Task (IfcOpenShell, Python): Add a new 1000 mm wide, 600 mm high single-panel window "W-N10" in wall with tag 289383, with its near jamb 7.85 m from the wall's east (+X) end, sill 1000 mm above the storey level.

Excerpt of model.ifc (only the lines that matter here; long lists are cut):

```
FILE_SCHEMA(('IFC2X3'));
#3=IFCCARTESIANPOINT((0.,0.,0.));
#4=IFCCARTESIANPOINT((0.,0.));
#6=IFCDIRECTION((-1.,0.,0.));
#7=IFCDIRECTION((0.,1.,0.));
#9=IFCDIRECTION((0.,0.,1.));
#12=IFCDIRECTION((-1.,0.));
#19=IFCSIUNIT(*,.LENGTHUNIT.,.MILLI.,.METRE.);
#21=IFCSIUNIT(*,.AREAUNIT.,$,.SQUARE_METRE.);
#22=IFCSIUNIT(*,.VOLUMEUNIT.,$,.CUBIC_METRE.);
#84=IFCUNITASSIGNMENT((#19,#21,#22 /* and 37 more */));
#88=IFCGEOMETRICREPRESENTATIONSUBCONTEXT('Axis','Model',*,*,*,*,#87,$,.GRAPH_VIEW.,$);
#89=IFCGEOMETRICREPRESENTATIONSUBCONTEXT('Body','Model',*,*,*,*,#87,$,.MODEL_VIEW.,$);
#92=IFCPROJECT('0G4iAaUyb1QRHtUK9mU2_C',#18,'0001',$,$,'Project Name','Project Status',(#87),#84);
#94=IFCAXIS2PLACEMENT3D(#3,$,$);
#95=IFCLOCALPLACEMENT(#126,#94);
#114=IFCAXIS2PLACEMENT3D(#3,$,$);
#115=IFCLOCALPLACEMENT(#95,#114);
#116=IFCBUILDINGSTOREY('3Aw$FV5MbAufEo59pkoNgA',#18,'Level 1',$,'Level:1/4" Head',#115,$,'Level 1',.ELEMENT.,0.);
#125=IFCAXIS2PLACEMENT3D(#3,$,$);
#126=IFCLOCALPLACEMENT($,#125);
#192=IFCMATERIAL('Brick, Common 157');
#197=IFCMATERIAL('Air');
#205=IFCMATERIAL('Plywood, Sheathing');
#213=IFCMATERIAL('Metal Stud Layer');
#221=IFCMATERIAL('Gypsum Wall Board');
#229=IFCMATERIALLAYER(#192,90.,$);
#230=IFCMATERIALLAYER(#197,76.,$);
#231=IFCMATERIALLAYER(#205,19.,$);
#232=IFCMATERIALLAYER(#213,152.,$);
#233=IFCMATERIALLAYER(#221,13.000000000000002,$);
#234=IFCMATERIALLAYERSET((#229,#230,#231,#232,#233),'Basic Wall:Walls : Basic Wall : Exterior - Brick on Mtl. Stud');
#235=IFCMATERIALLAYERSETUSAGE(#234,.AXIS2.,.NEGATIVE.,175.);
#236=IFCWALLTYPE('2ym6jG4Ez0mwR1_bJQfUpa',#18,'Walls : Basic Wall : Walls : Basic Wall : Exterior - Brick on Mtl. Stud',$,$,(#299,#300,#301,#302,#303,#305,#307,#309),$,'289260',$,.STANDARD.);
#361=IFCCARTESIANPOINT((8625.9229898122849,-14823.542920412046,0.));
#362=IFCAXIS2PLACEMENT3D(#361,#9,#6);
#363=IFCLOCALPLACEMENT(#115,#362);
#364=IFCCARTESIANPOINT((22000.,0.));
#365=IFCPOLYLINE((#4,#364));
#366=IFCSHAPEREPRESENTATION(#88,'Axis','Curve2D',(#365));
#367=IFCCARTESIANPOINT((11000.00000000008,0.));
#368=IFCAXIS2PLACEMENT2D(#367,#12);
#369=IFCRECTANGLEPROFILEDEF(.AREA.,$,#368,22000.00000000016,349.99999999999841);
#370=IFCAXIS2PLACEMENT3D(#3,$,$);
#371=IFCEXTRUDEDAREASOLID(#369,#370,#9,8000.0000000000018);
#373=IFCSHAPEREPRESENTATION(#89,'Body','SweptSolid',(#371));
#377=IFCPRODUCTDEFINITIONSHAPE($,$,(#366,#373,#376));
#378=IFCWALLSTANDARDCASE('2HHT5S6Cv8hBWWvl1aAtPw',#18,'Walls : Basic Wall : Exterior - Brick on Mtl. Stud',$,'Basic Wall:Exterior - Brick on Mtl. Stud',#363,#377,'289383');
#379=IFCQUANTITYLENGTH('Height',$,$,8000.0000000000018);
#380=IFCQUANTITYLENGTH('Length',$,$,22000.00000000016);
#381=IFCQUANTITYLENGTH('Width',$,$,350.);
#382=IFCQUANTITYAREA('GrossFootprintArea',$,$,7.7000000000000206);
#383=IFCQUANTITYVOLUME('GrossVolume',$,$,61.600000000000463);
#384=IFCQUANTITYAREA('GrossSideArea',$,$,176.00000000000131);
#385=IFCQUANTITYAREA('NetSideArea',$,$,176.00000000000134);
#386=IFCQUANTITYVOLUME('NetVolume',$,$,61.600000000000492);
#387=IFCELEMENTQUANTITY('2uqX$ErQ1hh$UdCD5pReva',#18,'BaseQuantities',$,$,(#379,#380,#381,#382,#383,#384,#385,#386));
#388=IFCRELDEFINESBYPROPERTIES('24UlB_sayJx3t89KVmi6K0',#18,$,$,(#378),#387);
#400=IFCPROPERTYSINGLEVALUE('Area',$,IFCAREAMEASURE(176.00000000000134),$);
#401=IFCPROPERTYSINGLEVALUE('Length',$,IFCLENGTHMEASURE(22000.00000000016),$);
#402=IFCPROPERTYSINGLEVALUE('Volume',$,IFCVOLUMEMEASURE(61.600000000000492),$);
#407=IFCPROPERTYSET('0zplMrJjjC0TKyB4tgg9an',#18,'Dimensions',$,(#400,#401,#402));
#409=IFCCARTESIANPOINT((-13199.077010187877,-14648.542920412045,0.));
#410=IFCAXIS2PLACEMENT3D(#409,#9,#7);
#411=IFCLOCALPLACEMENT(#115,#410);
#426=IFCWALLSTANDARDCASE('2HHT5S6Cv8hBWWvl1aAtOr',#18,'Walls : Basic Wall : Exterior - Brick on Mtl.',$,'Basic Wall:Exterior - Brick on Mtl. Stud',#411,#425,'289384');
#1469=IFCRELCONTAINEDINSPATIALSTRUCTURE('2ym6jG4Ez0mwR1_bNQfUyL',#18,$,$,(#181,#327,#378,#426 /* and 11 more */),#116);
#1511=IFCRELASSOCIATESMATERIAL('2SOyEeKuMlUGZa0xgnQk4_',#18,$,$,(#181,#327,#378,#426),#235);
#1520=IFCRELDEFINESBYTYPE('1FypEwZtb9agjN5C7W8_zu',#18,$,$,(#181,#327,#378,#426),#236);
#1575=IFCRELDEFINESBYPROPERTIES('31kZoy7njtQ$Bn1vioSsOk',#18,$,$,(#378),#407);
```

```python
import numpy as np
import ifcopenshell
import ifcopenshell.api.feature
import ifcopenshell.api.geometry
import ifcopenshell.api.pset
import ifcopenshell.api.root
import ifcopenshell.api.spatial
import ifcopenshell.api.type
import ifcopenshell.geom
import ifcopenshell.util.element
import ifcopenshell.util.placement
import ifcopenshell.util.representation
import ifcopenshell.util.shape
import ifcopenshell.util.unit

model = ifcopenshell.open("model.ifc")
unit_scale = ifcopenshell.util.unit.calculate_unit_scale(model)
area_scale = ifcopenshell.util.unit.calculate_unit_scale(model, "AREAUNIT")
volume_scale = ifcopenshell.util.unit.calculate_unit_scale(model, "VOLUMEUNIT")
settings = ifcopenshell.geom.settings()


def volume(element):
    """Net volume in cubic metres, openings subtracted."""
    shape = ifcopenshell.geom.create_shape(settings, element)
    return ifcopenshell.util.shape.get_volume(shape.geometry)


wall = model.by_id(378)
storey = ifcopenshell.util.element.get_container(wall, ifc_class="IfcBuildingStorey")
context = ifcopenshell.util.representation.get_context(model, "Model", "Body", "MODEL_VIEW")
before = volume(wall)

width, height, from_end, sill = 1, 0.6, 7.85, 1  # metres

# The wall runs along its own X axis, and the end named is its -X end.
wall_shape = ifcopenshell.geom.create_shape(settings, wall)
x, y, z = ifcopenshell.util.shape.get_vertices(wall_shape.geometry).T
start = x.min() + from_end
face, thickness = float(y.min()), float(y.max() - y.min())
wall_matrix = ifcopenshell.util.placement.get_local_placement(wall.ObjectPlacement)
level = ifcopenshell.util.placement.get_local_placement(storey.ObjectPlacement)[2, 3]


def in_wall(x, y):
    """Placement at x, y metres in the wall's axes, at sill height."""
    matrix = wall_matrix.copy()
    matrix[:, 3] = wall_matrix @ np.array([x / unit_scale, y / unit_scale, 0.0, 1.0])
    matrix[2, 3] = level + sill / unit_scale
    return matrix


# Opening: a box that overshoots both wall faces by 50 mm.
opening = ifcopenshell.api.root.create_entity(model, ifc_class="IfcOpeningElement")
box = ifcopenshell.api.geometry.add_wall_representation(
    model, context=context, length=width, height=height, thickness=thickness + 0.1
)
ifcopenshell.api.geometry.assign_representation(model, product=opening, representation=box)
ifcopenshell.api.geometry.edit_object_placement(model, product=opening, matrix=in_wall(start, face - 0.05), is_si=False)
ifcopenshell.api.feature.add_feature(model, feature=opening, element=wall)

window = ifcopenshell.api.root.create_entity(model, ifc_class="IfcWindow", name="W-N10")
window.OverallWidth, window.OverallHeight = width / unit_scale, height / unit_scale
body = ifcopenshell.api.geometry.add_window_representation(
    model,
    context=context,
    overall_width=window.OverallWidth,
    overall_height=window.OverallHeight,
    partition_type="SINGLE_PANEL",
)
ifcopenshell.api.geometry.assign_representation(model, product=window, representation=body)
ifcopenshell.api.spatial.assign_container(model, products=[window], relating_structure=storey)
fills = ifcopenshell.api.feature.add_filling(model, opening=opening, element=window)
fills.OwnerHistory = window.OwnerHistory  # required in IFC2X3

# IFC2X3 keeps the operation on the window style.
style = ifcopenshell.api.root.create_entity(model, ifc_class="IfcWindowStyle", name="W-N10")
style.OperationType, style.ConstructionType = "SINGLE_PANEL", "NOTDEFINED"
style.ParameterTakesPrecedence = style.Sizeable = False
ifcopenshell.api.type.assign_type(model, related_objects=[window], relating_type=style)

# Centre the window in the wall's thickness.
ifcopenshell.api.geometry.edit_object_placement(model, product=window, matrix=in_wall(start, face), is_si=False)
window_shape = ifcopenshell.geom.create_shape(settings, window)
depth = ifcopenshell.util.shape.get_vertices(window_shape.geometry)[:, 1]
offset = face + thickness / 2 - (depth.min() + depth.max()) / 2
ifcopenshell.api.geometry.edit_object_placement(model, product=window, matrix=in_wall(start, offset), is_si=False)

after = volume(wall)

# Update the wall's stored quantities.
qto = model.by_id(ifcopenshell.util.element.get_pset(wall, "BaseQuantities", should_inherit=False)["id"])
ifcopenshell.api.pset.edit_qto(model, qto=qto, properties={
    "NetSideArea": after / thickness / area_scale,
    "NetVolume": after / volume_scale,
})
pset = model.by_id(ifcopenshell.util.element.get_pset(wall, "Dimensions", should_inherit=False)["id"])
ifcopenshell.api.pset.edit_pset(model, pset=pset, properties={
    "Area": model.create_entity("IfcAreaMeasure", after / thickness / area_scale),
    "Volume": model.create_entity("IfcVolumeMeasure", after / volume_scale),
})

print(f"wall volume {before:.3f} -> {after:.3f} m3")

model.write("model-out.ifc")
```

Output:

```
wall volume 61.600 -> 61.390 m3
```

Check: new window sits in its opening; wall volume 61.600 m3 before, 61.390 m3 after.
